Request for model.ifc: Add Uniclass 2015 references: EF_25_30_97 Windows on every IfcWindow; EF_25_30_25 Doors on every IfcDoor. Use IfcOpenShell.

First a look at what the model holds.

```python
import ifcopenshell

model = ifcopenshell.open("model.ifc")
print(model.schema)
print("classifications:", [c.Name for c in model.by_type("IfcClassification")])
for ifc_class in ("IfcDoor", "IfcRoof", "IfcStair", "IfcWall", "IfcWindow"):
    print(ifc_class, len(model.by_type(ifc_class)))
```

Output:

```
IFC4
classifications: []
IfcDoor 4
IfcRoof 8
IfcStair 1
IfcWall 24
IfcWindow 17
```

```python
import ifcopenshell
import ifcopenshell.api.classification

model = ifcopenshell.open("model.ifc")

system = ifcopenshell.api.classification.add_classification(model, classification="Uniclass 2015")

codes = {
    "IfcWindow": ("EF_25_30_97", "Windows"),
    "IfcDoor": ("EF_25_30_25", "Doors"),
}
for ifc_class, (code, name) in codes.items():
    products = model.by_type(ifc_class)
    ifcopenshell.api.classification.add_reference(
        model, products=products, classification=system, identification=code, name=name
    )
    print(code, len(products))

model.write("model_v2.ifc")
```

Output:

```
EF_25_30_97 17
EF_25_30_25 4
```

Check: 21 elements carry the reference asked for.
